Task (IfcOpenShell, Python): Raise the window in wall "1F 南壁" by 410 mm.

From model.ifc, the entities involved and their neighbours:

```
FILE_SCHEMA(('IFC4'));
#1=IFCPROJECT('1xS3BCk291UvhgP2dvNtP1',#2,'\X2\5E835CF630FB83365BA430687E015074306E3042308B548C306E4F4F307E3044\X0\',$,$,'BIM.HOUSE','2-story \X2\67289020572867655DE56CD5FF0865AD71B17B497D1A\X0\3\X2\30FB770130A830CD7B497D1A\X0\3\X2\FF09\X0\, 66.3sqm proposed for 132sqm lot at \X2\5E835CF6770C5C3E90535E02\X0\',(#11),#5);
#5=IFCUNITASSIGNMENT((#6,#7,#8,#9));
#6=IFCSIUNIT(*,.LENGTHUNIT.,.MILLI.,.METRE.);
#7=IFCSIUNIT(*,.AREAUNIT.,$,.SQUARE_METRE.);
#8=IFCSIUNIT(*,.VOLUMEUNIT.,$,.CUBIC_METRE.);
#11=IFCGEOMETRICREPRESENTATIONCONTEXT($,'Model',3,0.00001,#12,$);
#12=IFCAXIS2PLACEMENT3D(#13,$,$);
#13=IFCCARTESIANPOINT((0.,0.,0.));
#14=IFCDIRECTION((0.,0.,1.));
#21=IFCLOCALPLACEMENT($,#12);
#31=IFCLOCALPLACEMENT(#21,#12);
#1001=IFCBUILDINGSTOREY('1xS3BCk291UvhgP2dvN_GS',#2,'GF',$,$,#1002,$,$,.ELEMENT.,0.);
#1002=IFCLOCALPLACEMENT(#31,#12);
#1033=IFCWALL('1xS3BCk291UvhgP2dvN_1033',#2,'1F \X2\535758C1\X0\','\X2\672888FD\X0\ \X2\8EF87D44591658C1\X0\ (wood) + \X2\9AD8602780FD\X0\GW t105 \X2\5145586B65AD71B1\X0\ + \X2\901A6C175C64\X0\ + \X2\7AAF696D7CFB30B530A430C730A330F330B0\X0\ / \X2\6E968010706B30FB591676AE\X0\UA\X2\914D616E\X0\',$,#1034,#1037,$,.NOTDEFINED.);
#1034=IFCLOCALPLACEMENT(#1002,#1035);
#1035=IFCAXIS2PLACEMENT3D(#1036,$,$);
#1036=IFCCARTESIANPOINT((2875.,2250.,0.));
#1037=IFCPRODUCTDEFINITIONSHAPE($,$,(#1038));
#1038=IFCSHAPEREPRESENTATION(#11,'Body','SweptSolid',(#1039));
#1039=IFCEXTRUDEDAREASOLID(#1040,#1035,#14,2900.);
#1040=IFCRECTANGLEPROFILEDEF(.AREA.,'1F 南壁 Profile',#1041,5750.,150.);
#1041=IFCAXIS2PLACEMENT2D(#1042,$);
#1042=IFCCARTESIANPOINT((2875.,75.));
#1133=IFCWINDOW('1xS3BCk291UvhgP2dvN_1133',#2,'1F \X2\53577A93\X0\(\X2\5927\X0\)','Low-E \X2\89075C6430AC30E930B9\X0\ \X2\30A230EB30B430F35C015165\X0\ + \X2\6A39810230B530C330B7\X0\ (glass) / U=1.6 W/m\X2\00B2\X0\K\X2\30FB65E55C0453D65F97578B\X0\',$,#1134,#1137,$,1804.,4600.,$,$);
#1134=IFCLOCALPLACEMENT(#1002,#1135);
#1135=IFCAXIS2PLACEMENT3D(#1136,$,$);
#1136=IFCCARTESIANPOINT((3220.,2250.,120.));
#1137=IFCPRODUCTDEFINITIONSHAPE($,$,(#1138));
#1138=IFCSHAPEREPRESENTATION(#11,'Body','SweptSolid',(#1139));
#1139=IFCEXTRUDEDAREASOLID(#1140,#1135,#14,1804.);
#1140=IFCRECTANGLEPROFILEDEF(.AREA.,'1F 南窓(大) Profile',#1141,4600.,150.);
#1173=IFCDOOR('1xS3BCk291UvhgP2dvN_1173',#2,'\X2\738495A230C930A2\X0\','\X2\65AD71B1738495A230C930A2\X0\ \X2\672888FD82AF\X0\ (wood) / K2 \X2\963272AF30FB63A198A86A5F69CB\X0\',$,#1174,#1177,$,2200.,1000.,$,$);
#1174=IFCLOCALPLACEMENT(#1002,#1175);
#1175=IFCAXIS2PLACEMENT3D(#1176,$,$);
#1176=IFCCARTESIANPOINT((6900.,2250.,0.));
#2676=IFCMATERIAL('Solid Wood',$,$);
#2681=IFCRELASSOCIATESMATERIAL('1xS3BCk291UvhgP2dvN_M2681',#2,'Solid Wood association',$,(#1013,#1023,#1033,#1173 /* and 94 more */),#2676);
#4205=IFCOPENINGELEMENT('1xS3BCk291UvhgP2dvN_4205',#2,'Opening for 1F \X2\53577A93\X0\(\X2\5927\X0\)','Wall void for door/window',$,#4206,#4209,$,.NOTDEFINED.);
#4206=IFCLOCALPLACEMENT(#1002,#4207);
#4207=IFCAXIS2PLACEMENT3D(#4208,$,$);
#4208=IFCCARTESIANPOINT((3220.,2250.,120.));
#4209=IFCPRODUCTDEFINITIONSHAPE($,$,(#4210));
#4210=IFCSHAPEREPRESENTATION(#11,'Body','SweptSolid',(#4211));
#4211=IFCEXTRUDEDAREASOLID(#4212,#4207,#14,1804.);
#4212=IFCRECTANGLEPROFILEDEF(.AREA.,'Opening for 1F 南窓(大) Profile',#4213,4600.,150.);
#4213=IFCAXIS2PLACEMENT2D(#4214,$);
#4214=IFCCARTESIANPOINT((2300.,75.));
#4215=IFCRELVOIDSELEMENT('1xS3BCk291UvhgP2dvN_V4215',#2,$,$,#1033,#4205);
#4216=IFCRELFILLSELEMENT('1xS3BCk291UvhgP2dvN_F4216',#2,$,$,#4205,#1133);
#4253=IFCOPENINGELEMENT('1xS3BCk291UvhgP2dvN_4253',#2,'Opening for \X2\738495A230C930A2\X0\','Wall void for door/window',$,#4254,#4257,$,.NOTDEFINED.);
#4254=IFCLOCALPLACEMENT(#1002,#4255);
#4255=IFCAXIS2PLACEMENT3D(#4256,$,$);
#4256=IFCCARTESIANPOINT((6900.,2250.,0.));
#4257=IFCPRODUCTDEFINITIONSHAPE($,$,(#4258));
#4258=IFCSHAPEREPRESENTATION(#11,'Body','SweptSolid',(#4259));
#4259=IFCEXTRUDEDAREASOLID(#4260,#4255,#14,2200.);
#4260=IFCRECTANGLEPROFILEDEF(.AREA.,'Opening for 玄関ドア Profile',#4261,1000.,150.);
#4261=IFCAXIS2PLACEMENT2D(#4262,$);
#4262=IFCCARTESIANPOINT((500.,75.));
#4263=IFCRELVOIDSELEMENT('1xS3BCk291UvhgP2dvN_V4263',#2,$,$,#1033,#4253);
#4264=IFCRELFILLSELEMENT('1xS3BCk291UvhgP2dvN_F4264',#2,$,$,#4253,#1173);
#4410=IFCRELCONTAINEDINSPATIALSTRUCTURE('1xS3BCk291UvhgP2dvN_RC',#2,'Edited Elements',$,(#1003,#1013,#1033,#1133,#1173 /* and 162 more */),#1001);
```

```python
import numpy as np
import ifcopenshell
import ifcopenshell.api.geometry
import ifcopenshell.util.placement
import ifcopenshell.util.unit

model = ifcopenshell.open("model.ifc")
unit_scale = ifcopenshell.util.unit.calculate_unit_scale(model)

window = model.by_guid("1xS3BCk291UvhgP2dvN_1133")
opening = window.FillsVoids[0].RelatingOpeningElement
dz = 0.41 / unit_scale

shift = np.array([0.0, 0.0, dz])
# The window is not placed relative to its opening, so move both.
for product in (opening, window):
    matrix = ifcopenshell.util.placement.get_local_placement(product.ObjectPlacement)
    matrix[:3, 3] += shift
    ifcopenshell.api.geometry.edit_object_placement(model, product=product, matrix=matrix, is_si=False)

print(f"moved by {dz * unit_scale:+.3f} m")

model.write("model_v2.ifc")
```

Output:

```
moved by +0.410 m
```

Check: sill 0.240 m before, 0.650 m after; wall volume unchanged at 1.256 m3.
